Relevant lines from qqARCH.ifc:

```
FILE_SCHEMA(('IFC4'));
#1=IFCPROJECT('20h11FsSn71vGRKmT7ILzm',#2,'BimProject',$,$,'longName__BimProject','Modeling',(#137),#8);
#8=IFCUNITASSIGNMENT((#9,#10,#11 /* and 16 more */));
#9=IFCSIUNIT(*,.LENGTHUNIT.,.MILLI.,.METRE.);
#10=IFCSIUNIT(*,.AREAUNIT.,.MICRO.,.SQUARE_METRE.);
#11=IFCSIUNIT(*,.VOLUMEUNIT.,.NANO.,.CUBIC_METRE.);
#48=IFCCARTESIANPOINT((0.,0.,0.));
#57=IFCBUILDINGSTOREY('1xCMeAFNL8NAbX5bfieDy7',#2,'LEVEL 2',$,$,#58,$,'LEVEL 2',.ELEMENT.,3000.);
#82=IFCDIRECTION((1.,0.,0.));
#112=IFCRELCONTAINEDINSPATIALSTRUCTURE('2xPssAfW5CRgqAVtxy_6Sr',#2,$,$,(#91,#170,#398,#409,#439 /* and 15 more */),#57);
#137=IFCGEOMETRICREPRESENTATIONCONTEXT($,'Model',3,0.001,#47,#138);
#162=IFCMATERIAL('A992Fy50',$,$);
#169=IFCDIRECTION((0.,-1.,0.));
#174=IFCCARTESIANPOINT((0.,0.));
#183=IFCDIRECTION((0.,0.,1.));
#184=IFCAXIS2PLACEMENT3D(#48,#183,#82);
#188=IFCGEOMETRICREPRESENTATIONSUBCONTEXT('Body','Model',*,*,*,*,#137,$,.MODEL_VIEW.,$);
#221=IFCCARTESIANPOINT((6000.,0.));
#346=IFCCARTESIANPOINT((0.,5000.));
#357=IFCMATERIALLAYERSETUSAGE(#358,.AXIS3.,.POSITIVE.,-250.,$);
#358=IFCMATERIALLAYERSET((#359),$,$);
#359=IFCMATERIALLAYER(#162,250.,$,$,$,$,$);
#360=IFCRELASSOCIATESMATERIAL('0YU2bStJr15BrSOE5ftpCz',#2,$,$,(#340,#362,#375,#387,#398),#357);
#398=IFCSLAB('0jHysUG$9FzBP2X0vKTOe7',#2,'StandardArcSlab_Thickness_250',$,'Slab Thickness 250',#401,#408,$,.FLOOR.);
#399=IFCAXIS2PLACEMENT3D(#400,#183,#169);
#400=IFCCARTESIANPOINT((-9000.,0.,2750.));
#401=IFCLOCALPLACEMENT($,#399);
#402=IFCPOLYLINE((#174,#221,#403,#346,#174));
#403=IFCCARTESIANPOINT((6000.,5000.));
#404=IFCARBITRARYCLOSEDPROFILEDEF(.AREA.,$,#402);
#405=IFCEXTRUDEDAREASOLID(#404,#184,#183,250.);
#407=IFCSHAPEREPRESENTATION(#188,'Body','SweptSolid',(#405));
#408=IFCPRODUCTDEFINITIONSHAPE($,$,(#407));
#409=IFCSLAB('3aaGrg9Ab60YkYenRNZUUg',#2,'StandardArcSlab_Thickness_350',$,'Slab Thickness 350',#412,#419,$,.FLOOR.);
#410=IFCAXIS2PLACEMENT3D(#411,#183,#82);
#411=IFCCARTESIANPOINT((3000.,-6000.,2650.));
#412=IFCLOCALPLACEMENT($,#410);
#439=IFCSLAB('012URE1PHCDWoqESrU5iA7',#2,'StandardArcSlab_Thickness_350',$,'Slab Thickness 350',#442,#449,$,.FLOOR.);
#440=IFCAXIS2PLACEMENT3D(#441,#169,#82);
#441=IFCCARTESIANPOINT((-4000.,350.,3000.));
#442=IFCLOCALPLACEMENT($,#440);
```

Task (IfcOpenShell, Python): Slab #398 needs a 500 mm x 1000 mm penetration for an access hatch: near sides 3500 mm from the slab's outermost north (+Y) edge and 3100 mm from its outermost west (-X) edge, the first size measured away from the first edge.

```python
import numpy as np
import ifcopenshell
import ifcopenshell.api.feature
import ifcopenshell.api.geometry
import ifcopenshell.api.root
import ifcopenshell.geom
import ifcopenshell.util.placement
import ifcopenshell.util.representation
import ifcopenshell.util.shape
import ifcopenshell.util.unit

model = ifcopenshell.open("qqARCH.ifc")
unit_scale = ifcopenshell.util.unit.calculate_unit_scale(model)
settings = ifcopenshell.geom.settings()


def volume(element):
    """Net volume in cubic metres, openings subtracted."""
    shape = ifcopenshell.geom.create_shape(settings, element)
    return ifcopenshell.util.shape.get_volume(shape.geometry)


slab = model.by_guid("0jHysUG$9FzBP2X0vKTOe7")
before = volume(slab)

# Extent in the slab's own axes, in metres. The edges named are its -X and -Y sides.
slab_shape = ifcopenshell.geom.create_shape(settings, slab)
vertices = ifcopenshell.util.shape.get_vertices(slab_shape.geometry)
x_min, y_min, bottom = vertices.min(axis=0)
top = vertices[:, 2].max()

opening = ifcopenshell.api.root.create_entity(model, ifc_class="IfcOpeningElement", name="Access hatch opening", predefined_type="OPENING")
context = ifcopenshell.util.representation.get_context(model, "Model", "Body", "MODEL_VIEW")
width, depth = 0.5, 1
outline = [(0.0, 0.0), (width, 0.0), (width, depth), (0.0, depth), (0.0, 0.0)]
# Overshoot both faces by 50 mm so the cut is clean.
shape = ifcopenshell.api.geometry.add_slab_representation(
    model, context=context, depth=top - bottom + 0.1, polyline=outline
)
ifcopenshell.api.geometry.assign_representation(model, product=opening, representation=shape)

matrix = ifcopenshell.util.placement.get_local_placement(slab.ObjectPlacement)
matrix[:, 3] = matrix @ np.append(np.array([x_min + 3.5, y_min + 3.1, bottom - 0.05]) / unit_scale, 1.0)
ifcopenshell.api.geometry.edit_object_placement(model, product=opening, matrix=matrix, is_si=False)
ifcopenshell.api.feature.add_feature(model, feature=opening, element=slab)

after = volume(slab)

print(f"slab volume {before:.3f} -> {after:.3f} m3")

model.write("qqARCH_edited.ifc")
```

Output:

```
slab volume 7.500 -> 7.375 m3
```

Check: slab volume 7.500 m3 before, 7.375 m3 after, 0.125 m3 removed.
